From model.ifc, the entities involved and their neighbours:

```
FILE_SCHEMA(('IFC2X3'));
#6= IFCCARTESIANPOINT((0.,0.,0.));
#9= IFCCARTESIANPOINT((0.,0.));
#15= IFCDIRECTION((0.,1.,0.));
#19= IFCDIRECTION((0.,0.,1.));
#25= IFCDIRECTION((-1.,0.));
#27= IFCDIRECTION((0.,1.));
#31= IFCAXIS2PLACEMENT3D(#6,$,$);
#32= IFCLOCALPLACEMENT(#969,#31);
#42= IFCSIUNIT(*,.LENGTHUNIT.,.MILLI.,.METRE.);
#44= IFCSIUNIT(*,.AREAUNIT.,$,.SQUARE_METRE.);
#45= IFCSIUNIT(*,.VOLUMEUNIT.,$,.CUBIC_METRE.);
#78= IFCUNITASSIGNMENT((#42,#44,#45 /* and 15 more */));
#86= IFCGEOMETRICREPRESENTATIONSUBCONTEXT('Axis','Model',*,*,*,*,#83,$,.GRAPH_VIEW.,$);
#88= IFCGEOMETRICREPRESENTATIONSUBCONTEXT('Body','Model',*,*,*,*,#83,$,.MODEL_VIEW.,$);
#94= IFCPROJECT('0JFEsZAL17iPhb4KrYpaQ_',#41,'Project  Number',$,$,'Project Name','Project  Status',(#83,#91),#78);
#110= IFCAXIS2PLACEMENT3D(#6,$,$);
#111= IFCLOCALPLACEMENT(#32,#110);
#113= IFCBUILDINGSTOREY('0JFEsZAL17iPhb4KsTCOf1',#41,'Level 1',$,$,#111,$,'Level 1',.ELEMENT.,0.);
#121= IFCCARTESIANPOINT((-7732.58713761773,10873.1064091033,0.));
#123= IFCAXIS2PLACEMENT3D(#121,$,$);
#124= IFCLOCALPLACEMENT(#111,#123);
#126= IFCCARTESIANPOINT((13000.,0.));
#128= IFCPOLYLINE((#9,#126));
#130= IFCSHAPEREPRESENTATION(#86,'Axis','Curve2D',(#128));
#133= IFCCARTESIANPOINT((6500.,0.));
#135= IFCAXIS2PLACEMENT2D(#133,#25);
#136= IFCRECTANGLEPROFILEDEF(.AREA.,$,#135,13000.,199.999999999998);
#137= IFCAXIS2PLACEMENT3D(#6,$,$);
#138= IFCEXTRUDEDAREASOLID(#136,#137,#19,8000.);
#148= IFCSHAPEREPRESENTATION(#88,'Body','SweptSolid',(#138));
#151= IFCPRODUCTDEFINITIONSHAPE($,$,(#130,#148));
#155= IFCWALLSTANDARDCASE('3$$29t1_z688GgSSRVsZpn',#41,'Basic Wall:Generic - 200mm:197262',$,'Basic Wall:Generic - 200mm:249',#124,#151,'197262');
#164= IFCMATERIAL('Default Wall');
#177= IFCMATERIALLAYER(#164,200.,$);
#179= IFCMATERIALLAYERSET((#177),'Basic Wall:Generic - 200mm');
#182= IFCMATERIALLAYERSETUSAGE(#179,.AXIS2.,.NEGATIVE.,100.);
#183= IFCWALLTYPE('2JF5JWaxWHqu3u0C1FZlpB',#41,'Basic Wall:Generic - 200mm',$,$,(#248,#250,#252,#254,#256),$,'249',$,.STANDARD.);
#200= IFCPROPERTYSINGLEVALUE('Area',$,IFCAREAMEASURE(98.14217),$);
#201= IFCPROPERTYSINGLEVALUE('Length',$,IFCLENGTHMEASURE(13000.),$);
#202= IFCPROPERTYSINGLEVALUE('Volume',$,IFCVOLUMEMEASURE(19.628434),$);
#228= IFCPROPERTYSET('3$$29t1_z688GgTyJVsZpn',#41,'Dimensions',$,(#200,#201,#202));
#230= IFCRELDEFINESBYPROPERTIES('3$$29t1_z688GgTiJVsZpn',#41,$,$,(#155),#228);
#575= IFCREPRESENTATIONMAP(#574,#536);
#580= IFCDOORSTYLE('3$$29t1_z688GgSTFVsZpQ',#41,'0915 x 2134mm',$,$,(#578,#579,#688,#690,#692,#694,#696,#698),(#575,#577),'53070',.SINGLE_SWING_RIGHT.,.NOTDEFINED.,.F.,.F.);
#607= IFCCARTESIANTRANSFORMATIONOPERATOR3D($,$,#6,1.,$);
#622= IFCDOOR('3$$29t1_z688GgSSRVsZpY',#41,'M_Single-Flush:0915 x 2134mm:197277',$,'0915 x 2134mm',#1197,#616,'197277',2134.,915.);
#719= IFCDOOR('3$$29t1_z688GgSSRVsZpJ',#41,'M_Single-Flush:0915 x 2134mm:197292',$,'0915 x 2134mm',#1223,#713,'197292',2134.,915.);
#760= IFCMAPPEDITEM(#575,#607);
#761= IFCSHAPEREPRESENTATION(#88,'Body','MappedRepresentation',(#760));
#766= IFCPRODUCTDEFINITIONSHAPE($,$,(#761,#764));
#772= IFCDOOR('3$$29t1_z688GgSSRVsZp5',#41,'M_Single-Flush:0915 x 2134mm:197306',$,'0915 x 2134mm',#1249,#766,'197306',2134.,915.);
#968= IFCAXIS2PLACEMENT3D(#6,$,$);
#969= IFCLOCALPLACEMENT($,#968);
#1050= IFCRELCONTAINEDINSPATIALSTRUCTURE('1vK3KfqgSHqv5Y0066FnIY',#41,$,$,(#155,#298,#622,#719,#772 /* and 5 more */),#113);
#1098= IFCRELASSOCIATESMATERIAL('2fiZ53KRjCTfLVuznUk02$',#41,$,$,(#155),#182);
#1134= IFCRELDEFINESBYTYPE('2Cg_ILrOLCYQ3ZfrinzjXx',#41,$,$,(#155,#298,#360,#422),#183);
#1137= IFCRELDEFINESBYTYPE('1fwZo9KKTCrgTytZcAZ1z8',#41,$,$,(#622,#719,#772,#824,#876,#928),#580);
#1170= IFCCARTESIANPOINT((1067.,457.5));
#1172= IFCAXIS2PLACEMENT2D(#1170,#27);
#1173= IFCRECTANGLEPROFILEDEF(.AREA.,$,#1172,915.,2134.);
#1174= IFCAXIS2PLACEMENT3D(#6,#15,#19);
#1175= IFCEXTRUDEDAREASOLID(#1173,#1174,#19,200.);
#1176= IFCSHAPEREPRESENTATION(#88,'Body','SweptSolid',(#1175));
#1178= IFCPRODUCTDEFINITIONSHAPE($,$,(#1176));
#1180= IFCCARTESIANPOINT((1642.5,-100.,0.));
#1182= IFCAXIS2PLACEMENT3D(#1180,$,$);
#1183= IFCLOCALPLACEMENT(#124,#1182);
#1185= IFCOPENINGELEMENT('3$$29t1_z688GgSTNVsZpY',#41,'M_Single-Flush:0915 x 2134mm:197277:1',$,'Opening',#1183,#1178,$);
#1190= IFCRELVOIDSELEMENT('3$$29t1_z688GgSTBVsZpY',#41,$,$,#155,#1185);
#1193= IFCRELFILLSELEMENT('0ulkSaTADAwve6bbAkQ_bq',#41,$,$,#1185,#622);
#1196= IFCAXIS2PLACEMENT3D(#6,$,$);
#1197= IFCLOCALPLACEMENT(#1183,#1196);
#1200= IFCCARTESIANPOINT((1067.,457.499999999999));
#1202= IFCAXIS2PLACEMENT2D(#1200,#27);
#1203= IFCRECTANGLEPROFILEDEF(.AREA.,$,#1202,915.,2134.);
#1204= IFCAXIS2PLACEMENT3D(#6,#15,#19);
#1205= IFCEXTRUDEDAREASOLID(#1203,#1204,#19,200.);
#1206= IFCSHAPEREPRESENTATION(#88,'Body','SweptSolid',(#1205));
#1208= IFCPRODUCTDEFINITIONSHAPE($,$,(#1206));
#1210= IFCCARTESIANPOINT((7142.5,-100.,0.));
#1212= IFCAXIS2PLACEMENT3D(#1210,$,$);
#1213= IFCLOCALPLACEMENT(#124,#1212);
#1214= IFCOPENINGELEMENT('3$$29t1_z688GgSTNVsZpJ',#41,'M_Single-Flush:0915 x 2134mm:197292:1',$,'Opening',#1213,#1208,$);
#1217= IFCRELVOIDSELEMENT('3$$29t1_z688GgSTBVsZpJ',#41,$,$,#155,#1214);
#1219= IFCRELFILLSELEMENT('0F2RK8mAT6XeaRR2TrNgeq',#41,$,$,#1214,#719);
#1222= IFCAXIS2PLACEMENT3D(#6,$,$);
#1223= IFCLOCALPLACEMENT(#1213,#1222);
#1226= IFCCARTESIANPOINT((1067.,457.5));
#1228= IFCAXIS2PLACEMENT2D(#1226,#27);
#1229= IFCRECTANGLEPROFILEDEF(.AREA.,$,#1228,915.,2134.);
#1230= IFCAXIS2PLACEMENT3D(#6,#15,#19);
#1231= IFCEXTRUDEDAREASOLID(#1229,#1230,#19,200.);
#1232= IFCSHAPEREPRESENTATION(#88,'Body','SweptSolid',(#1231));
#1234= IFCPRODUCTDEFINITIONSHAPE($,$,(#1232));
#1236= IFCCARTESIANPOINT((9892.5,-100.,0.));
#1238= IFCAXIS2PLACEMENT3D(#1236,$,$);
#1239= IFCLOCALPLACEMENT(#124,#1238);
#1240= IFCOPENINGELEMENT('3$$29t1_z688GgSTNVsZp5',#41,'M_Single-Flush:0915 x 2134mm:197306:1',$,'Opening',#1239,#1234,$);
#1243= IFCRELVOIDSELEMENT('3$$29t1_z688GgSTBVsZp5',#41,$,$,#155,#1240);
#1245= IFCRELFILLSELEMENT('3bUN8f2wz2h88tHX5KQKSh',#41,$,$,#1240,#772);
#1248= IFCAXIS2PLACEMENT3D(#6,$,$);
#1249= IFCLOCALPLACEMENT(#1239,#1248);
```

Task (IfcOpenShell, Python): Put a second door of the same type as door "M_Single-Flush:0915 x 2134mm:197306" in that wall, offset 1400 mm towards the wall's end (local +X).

```python
import ifcopenshell
import ifcopenshell.api.feature
import ifcopenshell.api.geometry
import ifcopenshell.api.pset
import ifcopenshell.api.root
import ifcopenshell.geom
import ifcopenshell.util.element
import ifcopenshell.util.placement
import ifcopenshell.util.shape
import ifcopenshell.util.unit

model = ifcopenshell.open("model.ifc")
unit_scale = ifcopenshell.util.unit.calculate_unit_scale(model)
area_scale = ifcopenshell.util.unit.calculate_unit_scale(model, "AREAUNIT")
volume_scale = ifcopenshell.util.unit.calculate_unit_scale(model, "VOLUMEUNIT")
settings = ifcopenshell.geom.settings()


def volume(element):
    """Net volume in cubic metres, openings subtracted."""
    shape = ifcopenshell.geom.create_shape(settings, element)
    return ifcopenshell.util.shape.get_volume(shape.geometry)


def reuse_history(source, copy):
    """copy_class also copies each property set's owner history, people and application; keep the originals."""
    for rel in copy.IsDefinedBy:
        if rel.is_a("IfcRelDefinesByProperties") and (history := rel.RelatingPropertyDefinition.OwnerHistory):
            rel.RelatingPropertyDefinition.OwnerHistory = source.OwnerHistory
            ifcopenshell.util.element.remove_deep2(model, history)


door = model.by_guid("3$$29t1_z688GgSSRVsZp5")
opening = door.FillsVoids[0].RelatingOpeningElement
wall = opening.VoidsElements[0].RelatingBuildingElement
before = volume(wall)
shift = ifcopenshell.util.placement.get_local_placement(wall.ObjectPlacement)[:3, 0] * 1.4 / unit_scale

# copy_class copies the void relationship, type, container and properties, but no geometry.
new_opening = ifcopenshell.api.root.copy_class(model, product=opening)
new_opening.Representation = ifcopenshell.util.element.copy_deep(
    model, opening.Representation, exclude=["IfcGeometricRepresentationContext", "IfcRepresentationMap"]
)
new_opening.Name = "M_Single-Flush:0915 x 2134mm"
new_door = ifcopenshell.api.root.copy_class(model, product=door)
new_door.Representation = ifcopenshell.util.element.copy_deep(
    model, door.Representation, exclude=["IfcGeometricRepresentationContext", "IfcRepresentationMap"]
)
new_door.Name = "M_Single-Flush:0915 x 2134mm"
new_door.Tag = None
reuse_history(door, new_door)
fills = ifcopenshell.api.feature.add_filling(model, opening=new_opening, element=new_door)
fills.OwnerHistory = new_door.OwnerHistory  # required in IFC2X3

for old, new in ((opening, new_opening), (door, new_door)):
    matrix = ifcopenshell.util.placement.get_local_placement(old.ObjectPlacement)
    matrix[:3, 3] += shift
    ifcopenshell.api.geometry.edit_object_placement(model, product=new, matrix=matrix, is_si=False)

after = volume(wall)
thickness = 0.2  # wall thickness in metres

# Update the wall's stored quantities.
pset = model.by_id(ifcopenshell.util.element.get_pset(wall, "Dimensions", should_inherit=False)["id"])
ifcopenshell.api.pset.edit_pset(model, pset=pset, properties={
    "Area": model.create_entity("IfcAreaMeasure", after / thickness / area_scale),
    "Volume": model.create_entity("IfcVolumeMeasure", after / volume_scale),
})

print(f"wall volume {before:.3f} -> {after:.3f} m3")

model.write("model_edited.ifc")
```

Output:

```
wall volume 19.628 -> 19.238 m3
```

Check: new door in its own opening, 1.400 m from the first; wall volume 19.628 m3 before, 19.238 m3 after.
